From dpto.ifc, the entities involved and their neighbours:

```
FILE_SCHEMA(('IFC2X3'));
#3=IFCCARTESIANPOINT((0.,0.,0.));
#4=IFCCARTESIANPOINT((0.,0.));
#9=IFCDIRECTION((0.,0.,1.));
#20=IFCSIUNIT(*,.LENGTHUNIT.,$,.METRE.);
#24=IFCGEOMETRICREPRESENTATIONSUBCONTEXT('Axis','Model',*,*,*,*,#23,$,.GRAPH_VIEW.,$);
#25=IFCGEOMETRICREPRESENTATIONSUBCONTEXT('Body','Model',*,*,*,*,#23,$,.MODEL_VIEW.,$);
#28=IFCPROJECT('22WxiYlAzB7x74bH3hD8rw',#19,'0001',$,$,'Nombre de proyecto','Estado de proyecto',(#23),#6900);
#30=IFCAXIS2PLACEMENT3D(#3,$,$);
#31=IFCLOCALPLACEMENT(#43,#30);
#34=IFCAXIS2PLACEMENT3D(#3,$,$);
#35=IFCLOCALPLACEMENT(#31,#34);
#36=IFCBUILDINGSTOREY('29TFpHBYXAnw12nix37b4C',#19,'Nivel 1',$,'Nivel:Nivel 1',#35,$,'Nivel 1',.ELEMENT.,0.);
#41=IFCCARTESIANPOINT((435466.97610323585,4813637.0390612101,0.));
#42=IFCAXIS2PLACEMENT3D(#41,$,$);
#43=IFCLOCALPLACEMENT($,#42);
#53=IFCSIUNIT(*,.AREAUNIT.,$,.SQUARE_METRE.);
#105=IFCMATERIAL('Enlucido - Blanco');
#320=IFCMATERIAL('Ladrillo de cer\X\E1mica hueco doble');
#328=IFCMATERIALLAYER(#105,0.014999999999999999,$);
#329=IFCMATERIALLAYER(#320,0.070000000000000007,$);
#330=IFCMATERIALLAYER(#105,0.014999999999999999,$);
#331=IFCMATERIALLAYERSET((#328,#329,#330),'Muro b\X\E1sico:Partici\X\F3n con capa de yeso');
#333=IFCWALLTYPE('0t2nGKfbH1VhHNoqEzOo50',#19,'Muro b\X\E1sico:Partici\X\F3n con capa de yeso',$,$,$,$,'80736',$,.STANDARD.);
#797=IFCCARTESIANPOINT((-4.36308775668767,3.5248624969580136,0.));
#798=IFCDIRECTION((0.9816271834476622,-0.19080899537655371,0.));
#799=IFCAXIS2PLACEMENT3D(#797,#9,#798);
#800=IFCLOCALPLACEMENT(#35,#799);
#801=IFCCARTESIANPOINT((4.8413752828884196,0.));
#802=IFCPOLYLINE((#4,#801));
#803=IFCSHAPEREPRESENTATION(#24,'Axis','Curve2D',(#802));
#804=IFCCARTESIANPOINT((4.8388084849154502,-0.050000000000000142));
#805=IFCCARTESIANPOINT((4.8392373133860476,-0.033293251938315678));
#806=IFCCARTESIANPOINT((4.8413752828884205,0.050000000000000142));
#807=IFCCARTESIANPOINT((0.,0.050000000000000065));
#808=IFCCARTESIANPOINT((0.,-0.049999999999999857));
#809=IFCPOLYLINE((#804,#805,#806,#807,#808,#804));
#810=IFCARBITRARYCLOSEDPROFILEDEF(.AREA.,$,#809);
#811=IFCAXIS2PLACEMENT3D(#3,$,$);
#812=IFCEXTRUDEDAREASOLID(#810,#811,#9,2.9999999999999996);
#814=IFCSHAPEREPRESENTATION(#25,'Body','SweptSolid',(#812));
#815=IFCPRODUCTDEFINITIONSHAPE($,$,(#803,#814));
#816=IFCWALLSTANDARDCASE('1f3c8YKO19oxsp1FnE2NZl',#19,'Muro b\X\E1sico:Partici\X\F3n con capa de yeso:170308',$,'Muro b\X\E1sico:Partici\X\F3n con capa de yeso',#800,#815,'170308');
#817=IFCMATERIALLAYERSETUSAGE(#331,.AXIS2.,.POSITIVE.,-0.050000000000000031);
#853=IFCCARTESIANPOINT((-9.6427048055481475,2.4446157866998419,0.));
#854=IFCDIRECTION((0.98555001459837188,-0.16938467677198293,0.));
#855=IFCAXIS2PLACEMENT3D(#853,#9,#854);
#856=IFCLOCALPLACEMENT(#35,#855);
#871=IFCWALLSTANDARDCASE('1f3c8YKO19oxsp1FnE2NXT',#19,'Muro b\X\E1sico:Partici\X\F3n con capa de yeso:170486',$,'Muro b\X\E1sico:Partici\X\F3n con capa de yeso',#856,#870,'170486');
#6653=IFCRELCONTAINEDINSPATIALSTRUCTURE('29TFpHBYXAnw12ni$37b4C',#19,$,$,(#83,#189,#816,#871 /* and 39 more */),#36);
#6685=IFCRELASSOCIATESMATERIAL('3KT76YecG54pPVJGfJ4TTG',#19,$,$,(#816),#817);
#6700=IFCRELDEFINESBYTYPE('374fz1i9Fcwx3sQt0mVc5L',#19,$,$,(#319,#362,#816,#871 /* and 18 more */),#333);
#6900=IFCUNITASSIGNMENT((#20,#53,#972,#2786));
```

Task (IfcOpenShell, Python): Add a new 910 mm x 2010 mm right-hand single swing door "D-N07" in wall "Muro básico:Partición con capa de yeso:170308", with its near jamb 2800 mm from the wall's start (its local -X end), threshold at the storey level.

```python
import numpy as np
import ifcopenshell
import ifcopenshell.api.feature
import ifcopenshell.api.geometry
import ifcopenshell.api.root
import ifcopenshell.api.spatial
import ifcopenshell.api.type
import ifcopenshell.geom
import ifcopenshell.util.element
import ifcopenshell.util.placement
import ifcopenshell.util.representation
import ifcopenshell.util.shape
import ifcopenshell.util.unit

model = ifcopenshell.open("dpto.ifc")
unit_scale = ifcopenshell.util.unit.calculate_unit_scale(model)
settings = ifcopenshell.geom.settings()


def volume(element):
    """Net volume in cubic metres, openings subtracted."""
    shape = ifcopenshell.geom.create_shape(settings, element)
    return ifcopenshell.util.shape.get_volume(shape.geometry)


wall = model.by_id(816)
storey = ifcopenshell.util.element.get_container(wall, ifc_class="IfcBuildingStorey")
context = ifcopenshell.util.representation.get_context(model, "Model", "Body", "MODEL_VIEW")
before = volume(wall)

width, height, from_end, sill = 0.91, 2.01, 2.8, 0.0  # metres

# The wall runs along its own X axis, and the end named is its -X end.
wall_shape = ifcopenshell.geom.create_shape(settings, wall)
x, y, z = ifcopenshell.util.shape.get_vertices(wall_shape.geometry).T
start = x.min() + from_end
face, thickness = float(y.min()), float(y.max() - y.min())
wall_matrix = ifcopenshell.util.placement.get_local_placement(wall.ObjectPlacement)
level = ifcopenshell.util.placement.get_local_placement(storey.ObjectPlacement)[2, 3]


def in_wall(x, y):
    """Placement at x, y metres in the wall's axes, at sill height."""
    matrix = wall_matrix.copy()
    matrix[:, 3] = wall_matrix @ np.array([x / unit_scale, y / unit_scale, 0.0, 1.0])
    matrix[2, 3] = level + sill / unit_scale
    return matrix


# Opening: a box that overshoots both wall faces by 50 mm.
opening = ifcopenshell.api.root.create_entity(model, ifc_class="IfcOpeningElement")
box = ifcopenshell.api.geometry.add_wall_representation(
    model, context=context, length=width, height=height, thickness=thickness + 0.1
)
ifcopenshell.api.geometry.assign_representation(model, product=opening, representation=box)
ifcopenshell.api.geometry.edit_object_placement(model, product=opening, matrix=in_wall(start, face - 0.05), is_si=False)
ifcopenshell.api.feature.add_feature(model, feature=opening, element=wall)

door = ifcopenshell.api.root.create_entity(model, ifc_class="IfcDoor", name="D-N07")
door.OverallWidth, door.OverallHeight = width / unit_scale, height / unit_scale
body = ifcopenshell.api.geometry.add_door_representation(
    model,
    context=context,
    overall_width=door.OverallWidth,
    overall_height=door.OverallHeight,
    operation_type="SINGLE_SWING_RIGHT",
    lining_properties={"LiningDepth": thickness / unit_scale, "ThresholdDepth": thickness / unit_scale},
)
ifcopenshell.api.geometry.assign_representation(model, product=door, representation=body)
ifcopenshell.api.spatial.assign_container(model, products=[door], relating_structure=storey)
fills = ifcopenshell.api.feature.add_filling(model, opening=opening, element=door)
fills.OwnerHistory = door.OwnerHistory  # required in IFC2X3

# IFC2X3 keeps the operation on the door style.
style = ifcopenshell.api.root.create_entity(model, ifc_class="IfcDoorStyle", name="D-N07")
style.OperationType, style.ConstructionType = "SINGLE_SWING_RIGHT", "NOTDEFINED"
style.ParameterTakesPrecedence = style.Sizeable = False
ifcopenshell.api.type.assign_type(model, related_objects=[door], relating_type=style)

# The lining spans the wall, so the door starts at the wall face.
ifcopenshell.api.geometry.edit_object_placement(model, product=door, matrix=in_wall(start, face), is_si=False)

after = volume(wall)

print(f"wall volume {before:.3f} -> {after:.3f} m3")

model.write("dpto_edited.ifc")
```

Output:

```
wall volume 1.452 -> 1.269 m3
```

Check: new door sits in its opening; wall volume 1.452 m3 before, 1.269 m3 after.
